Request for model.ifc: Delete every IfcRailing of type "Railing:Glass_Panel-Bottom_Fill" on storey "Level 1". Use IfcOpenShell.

First a look at what the model holds.

```python
import ifcopenshell
import ifcopenshell.util.element

model = ifcopenshell.open("model.ifc")
print(model.schema)
storey = next(s for s in model.by_type("IfcBuildingStorey") if s.Name == "Level 1")
railings = [e for e in ifcopenshell.util.element.get_decomposition(storey) if e.is_a("IfcRailing")]
seen = {}
for e in railings:
    element_type = ifcopenshell.util.element.get_type(e)
    name = element_type.Name if element_type not in (None, e) else None
    seen[name] = seen.get(name, 0) + 1
for name, count in sorted(seen.items(), key=str):
    print(count, "x", name)
```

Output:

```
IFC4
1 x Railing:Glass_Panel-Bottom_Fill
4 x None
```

```python
import ifcopenshell
import ifcopenshell.api.root
import ifcopenshell.util.element

model = ifcopenshell.open("model.ifc")

storey = next(s for s in model.by_type("IfcBuildingStorey") if s.Name == "Level 1")
railings = [e for e in ifcopenshell.util.element.get_decomposition(storey) if e.is_a("IfcRailing")]
targets = [e for e in railings if (t := ifcopenshell.util.element.get_type(e)) not in (None, e) and t.Name == "Railing:Glass_Panel-Bottom_Fill"]

for e in targets:
    ifcopenshell.api.root.remove_product(model, product=e)
print(len(targets), "removed")

model.write("model-out.ifc")
```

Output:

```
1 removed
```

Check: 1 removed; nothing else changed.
